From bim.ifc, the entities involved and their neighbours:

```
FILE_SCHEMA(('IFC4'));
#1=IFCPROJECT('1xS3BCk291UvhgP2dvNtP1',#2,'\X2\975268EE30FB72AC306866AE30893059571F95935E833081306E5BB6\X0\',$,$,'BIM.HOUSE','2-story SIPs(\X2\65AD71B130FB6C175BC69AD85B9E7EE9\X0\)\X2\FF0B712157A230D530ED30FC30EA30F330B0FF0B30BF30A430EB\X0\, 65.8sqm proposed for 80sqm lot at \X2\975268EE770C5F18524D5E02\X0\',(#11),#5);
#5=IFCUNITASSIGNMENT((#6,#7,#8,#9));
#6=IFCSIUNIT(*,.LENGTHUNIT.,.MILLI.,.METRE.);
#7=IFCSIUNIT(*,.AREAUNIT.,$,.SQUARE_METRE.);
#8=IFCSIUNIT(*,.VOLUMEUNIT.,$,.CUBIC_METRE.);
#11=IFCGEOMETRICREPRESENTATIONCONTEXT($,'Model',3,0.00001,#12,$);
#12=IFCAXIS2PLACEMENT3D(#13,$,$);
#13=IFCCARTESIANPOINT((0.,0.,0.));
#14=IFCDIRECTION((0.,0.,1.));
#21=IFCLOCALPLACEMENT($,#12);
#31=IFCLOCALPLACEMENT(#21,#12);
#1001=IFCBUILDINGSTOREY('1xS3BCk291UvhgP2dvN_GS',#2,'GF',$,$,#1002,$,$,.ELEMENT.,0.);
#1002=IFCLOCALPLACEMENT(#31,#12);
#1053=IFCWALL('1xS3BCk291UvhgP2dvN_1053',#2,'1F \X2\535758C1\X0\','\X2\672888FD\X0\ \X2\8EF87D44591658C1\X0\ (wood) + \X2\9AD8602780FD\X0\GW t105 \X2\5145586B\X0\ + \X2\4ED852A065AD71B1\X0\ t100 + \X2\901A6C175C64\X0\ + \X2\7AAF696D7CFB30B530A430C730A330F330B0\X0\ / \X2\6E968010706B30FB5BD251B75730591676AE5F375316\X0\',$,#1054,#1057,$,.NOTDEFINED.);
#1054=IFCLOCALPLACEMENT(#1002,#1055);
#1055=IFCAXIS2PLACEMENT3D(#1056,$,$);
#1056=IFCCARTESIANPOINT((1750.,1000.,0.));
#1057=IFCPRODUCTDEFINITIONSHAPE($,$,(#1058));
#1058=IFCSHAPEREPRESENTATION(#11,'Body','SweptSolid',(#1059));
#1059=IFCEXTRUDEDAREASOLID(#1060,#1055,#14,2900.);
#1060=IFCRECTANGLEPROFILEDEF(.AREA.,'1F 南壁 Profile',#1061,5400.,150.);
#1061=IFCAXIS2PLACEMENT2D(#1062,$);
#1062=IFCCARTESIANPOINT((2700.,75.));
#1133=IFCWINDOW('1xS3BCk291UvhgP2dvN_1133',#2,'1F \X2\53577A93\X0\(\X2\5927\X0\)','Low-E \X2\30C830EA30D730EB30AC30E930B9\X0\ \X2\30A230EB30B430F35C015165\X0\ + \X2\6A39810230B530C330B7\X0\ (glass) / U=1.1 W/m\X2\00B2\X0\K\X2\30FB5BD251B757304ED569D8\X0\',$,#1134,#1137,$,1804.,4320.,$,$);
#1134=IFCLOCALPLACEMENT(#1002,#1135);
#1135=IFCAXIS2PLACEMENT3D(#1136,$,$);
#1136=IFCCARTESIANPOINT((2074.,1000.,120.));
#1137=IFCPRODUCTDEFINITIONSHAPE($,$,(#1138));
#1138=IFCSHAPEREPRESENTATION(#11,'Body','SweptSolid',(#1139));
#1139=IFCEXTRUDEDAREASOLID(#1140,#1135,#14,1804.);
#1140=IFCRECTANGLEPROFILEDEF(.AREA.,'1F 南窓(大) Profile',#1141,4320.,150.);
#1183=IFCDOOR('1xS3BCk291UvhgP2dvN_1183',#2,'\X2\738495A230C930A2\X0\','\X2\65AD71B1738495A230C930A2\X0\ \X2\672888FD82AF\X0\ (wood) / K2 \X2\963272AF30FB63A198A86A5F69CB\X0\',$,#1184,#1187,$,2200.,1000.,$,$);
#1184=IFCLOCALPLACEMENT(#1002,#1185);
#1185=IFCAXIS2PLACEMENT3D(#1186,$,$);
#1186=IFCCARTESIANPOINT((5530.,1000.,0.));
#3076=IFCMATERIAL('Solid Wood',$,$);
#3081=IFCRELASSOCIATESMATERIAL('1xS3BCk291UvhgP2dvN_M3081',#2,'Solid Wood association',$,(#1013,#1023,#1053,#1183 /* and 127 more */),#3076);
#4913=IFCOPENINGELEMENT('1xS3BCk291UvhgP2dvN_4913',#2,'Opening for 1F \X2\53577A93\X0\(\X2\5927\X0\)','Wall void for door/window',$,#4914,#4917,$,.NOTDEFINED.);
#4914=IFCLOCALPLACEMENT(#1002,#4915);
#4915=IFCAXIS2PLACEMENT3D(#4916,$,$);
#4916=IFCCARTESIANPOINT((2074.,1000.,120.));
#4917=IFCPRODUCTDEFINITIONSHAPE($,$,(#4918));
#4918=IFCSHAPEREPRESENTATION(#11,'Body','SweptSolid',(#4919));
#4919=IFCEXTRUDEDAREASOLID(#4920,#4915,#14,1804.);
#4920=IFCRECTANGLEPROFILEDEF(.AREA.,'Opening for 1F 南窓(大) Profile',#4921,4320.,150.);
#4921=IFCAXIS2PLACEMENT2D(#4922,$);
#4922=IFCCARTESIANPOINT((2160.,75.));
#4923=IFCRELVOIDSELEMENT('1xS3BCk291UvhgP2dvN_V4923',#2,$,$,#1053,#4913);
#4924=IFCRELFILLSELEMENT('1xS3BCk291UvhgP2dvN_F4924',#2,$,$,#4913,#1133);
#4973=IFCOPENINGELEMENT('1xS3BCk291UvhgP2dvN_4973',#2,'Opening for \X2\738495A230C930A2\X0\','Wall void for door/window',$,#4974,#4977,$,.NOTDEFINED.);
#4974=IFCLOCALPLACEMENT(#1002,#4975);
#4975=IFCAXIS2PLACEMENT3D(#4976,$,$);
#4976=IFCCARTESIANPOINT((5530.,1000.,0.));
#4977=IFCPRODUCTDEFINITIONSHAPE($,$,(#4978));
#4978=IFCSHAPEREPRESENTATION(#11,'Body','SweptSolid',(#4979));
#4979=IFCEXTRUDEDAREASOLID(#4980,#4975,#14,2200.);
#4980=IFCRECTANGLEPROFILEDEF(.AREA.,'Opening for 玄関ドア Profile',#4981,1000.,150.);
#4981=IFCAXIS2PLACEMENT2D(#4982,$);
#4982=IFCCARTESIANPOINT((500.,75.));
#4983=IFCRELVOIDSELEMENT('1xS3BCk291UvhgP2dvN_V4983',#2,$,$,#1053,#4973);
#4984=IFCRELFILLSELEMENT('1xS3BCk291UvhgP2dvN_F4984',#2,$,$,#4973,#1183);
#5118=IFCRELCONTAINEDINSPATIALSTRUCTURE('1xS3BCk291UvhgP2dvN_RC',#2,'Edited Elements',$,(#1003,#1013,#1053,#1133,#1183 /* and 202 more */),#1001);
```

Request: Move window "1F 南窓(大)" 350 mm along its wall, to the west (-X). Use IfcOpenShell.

```python
import ifcopenshell
import ifcopenshell.api.geometry
import ifcopenshell.util.placement
import ifcopenshell.util.unit

model = ifcopenshell.open("bim.ifc")
unit_scale = ifcopenshell.util.unit.calculate_unit_scale(model)

window = model.by_id(1133)
opening = window.FillsVoids[0].RelatingOpeningElement
wall = opening.VoidsElements[0].RelatingBuildingElement

wall_matrix = ifcopenshell.util.placement.get_local_placement(wall.ObjectPlacement)
shift = wall_matrix[:3, 0] * -0.35 / unit_scale
before = ifcopenshell.util.placement.get_local_placement(window.ObjectPlacement)[:3, 3].copy()

# The window is not placed relative to its opening, so move both.
for product in (opening, window):
    matrix = ifcopenshell.util.placement.get_local_placement(product.ObjectPlacement)
    matrix[:3, 3] += shift
    ifcopenshell.api.geometry.edit_object_placement(model, product=product, matrix=matrix, is_si=False)

after = ifcopenshell.util.placement.get_local_placement(window.ObjectPlacement)[:3, 3]
print("window moved by", (after - before).round(3) + 0.0)

model.write("bim_v2.ifc")
```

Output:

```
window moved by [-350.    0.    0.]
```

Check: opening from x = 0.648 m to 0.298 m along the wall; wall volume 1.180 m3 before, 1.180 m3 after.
